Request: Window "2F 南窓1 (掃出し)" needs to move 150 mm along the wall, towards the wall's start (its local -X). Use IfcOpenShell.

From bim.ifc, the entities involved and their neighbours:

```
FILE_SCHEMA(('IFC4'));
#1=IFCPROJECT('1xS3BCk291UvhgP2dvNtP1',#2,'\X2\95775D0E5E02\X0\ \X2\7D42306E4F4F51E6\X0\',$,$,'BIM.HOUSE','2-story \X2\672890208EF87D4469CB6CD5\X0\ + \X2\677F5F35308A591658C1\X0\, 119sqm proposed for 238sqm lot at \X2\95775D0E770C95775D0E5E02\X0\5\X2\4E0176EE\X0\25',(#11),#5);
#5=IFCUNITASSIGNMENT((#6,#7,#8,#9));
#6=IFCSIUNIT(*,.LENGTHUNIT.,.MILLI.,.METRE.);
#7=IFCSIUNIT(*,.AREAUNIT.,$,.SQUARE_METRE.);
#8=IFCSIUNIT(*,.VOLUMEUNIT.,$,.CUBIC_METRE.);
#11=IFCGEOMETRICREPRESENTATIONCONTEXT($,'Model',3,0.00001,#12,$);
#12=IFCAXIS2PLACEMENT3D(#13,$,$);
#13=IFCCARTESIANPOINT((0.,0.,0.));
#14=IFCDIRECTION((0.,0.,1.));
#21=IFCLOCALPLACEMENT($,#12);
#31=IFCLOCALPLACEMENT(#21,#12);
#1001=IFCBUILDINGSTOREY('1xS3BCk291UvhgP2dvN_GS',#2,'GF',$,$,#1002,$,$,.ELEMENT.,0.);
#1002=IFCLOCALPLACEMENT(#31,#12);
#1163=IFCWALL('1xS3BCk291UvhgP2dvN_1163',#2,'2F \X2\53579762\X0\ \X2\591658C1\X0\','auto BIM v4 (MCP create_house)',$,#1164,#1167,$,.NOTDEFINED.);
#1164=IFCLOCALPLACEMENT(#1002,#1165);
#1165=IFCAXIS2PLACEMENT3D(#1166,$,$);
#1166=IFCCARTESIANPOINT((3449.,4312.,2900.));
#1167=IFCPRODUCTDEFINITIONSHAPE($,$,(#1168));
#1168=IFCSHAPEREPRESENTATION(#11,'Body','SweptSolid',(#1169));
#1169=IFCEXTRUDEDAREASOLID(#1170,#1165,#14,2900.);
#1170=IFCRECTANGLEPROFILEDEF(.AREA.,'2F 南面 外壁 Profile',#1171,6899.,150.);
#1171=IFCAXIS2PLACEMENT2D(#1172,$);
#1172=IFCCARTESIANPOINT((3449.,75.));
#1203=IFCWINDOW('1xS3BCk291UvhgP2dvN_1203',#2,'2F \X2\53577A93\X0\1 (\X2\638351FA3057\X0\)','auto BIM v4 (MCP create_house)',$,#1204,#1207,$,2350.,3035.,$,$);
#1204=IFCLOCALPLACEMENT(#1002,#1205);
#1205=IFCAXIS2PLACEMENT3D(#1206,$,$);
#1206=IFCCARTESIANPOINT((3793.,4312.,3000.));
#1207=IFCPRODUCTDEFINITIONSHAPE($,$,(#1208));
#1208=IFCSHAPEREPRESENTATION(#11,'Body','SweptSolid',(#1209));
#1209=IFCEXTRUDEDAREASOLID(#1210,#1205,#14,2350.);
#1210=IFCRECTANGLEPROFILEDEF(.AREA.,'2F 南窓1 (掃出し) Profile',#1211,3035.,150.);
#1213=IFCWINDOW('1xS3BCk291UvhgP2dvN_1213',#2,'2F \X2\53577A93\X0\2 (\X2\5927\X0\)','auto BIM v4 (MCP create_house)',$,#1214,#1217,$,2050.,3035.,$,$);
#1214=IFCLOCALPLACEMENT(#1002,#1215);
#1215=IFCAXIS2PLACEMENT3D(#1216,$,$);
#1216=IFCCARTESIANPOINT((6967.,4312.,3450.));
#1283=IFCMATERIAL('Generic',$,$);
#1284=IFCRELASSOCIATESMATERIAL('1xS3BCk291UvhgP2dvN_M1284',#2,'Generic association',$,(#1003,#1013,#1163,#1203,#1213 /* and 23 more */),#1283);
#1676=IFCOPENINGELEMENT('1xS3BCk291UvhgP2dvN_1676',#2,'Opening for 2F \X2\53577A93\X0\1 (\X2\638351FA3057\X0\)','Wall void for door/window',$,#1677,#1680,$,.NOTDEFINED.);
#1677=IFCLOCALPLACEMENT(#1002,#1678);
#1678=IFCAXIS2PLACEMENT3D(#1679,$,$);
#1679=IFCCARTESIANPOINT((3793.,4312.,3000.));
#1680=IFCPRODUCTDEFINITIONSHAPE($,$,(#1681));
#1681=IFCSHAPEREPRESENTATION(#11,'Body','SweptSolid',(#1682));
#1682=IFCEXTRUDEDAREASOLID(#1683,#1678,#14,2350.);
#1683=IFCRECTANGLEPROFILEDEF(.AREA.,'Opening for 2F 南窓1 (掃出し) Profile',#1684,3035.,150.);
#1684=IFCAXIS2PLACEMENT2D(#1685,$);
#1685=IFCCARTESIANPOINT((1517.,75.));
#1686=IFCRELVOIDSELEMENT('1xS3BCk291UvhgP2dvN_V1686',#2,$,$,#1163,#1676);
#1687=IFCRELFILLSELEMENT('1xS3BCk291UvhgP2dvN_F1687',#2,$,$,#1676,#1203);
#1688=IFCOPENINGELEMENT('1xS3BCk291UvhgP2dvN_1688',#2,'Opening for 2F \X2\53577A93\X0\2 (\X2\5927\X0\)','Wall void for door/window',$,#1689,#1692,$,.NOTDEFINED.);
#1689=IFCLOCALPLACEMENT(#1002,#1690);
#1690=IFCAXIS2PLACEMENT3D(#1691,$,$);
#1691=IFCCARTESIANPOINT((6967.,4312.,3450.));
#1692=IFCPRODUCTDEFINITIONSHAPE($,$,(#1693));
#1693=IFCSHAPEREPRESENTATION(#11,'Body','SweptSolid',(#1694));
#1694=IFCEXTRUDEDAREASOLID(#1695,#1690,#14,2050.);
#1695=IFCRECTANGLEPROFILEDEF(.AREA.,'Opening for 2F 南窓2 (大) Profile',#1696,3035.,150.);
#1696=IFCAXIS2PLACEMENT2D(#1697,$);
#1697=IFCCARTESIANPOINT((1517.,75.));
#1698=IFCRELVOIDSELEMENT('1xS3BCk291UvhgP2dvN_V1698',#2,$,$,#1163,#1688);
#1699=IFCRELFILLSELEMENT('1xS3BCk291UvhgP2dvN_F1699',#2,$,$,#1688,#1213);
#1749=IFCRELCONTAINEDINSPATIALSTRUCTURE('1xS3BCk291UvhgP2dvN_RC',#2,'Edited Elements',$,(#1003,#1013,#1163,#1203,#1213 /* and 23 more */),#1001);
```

```python
import ifcopenshell
import ifcopenshell.api.geometry
import ifcopenshell.util.placement
import ifcopenshell.util.unit

model = ifcopenshell.open("bim.ifc")
unit_scale = ifcopenshell.util.unit.calculate_unit_scale(model)

window = model.by_guid("1xS3BCk291UvhgP2dvN_1203")
opening = window.FillsVoids[0].RelatingOpeningElement
wall = opening.VoidsElements[0].RelatingBuildingElement

wall_matrix = ifcopenshell.util.placement.get_local_placement(wall.ObjectPlacement)
shift = wall_matrix[:3, 0] * -0.15 / unit_scale
before = ifcopenshell.util.placement.get_local_placement(window.ObjectPlacement)[:3, 3].copy()

# The window is not placed relative to its opening, so move both.
for product in (opening, window):
    matrix = ifcopenshell.util.placement.get_local_placement(product.ObjectPlacement)
    matrix[:3, 3] += shift
    ifcopenshell.api.geometry.edit_object_placement(model, product=product, matrix=matrix, is_si=False)

after = ifcopenshell.util.placement.get_local_placement(window.ObjectPlacement)[:3, 3]
print("window moved by", (after - before).round(3) + 0.0)

model.write("bim-out.ifc")
```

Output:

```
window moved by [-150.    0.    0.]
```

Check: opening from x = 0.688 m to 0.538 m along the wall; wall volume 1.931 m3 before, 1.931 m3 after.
